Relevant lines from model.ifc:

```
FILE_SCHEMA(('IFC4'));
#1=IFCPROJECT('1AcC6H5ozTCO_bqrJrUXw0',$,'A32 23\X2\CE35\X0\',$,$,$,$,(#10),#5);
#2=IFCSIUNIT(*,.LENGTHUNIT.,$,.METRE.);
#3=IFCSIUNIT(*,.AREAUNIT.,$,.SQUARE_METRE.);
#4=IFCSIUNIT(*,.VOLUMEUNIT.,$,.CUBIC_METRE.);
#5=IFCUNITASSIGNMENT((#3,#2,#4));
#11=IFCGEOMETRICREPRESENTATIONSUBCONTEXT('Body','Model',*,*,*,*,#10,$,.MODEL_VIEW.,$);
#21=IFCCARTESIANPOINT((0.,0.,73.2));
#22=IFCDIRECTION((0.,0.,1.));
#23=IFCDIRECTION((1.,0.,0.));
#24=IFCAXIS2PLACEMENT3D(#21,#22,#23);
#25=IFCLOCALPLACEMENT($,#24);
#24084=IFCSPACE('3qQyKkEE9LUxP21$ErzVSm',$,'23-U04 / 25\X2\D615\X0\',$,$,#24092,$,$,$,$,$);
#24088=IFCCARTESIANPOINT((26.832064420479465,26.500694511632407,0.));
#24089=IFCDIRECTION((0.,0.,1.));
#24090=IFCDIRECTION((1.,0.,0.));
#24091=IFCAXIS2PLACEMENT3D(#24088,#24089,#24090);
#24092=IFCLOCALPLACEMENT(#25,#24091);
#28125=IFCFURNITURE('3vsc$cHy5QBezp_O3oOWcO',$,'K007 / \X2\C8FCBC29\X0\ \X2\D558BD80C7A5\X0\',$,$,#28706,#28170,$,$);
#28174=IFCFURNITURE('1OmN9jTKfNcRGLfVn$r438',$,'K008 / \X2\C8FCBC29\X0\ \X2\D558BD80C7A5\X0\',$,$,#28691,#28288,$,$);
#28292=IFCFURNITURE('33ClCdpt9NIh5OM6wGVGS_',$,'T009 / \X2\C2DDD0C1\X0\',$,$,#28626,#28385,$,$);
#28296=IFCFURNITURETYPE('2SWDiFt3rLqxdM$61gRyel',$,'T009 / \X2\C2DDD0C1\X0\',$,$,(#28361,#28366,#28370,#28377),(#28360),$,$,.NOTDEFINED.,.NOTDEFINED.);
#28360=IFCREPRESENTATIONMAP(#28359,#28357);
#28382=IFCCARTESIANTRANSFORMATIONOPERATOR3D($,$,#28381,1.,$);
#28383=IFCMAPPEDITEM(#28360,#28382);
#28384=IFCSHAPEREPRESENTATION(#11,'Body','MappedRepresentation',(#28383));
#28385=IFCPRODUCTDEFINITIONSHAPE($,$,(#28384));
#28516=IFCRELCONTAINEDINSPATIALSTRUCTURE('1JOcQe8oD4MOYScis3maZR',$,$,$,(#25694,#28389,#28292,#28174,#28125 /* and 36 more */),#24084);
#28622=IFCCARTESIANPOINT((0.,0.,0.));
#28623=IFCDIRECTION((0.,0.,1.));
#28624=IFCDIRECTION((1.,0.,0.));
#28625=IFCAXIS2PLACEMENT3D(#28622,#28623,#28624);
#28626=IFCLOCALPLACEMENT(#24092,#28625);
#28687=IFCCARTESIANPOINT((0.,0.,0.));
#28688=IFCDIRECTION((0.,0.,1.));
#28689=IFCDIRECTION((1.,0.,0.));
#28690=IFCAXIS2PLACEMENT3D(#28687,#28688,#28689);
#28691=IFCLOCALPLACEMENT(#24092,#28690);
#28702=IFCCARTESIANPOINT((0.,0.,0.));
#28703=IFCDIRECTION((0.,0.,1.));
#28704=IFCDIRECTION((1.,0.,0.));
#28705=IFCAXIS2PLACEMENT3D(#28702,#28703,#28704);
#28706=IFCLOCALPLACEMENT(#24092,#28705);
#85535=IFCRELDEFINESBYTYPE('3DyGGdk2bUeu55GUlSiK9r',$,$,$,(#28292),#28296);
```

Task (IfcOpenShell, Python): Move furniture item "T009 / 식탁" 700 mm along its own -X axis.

```python
import ifcopenshell
import ifcopenshell.api.geometry
import ifcopenshell.util.placement
import ifcopenshell.util.unit

model = ifcopenshell.open("model.ifc")
unit_scale = ifcopenshell.util.unit.calculate_unit_scale(model)

item = model.by_guid("33ClCdpt9NIh5OM6wGVGS_")
matrix = ifcopenshell.util.placement.get_local_placement(item.ObjectPlacement)
matrix[:3, 3] -= matrix[:3, 0] * 0.7 / unit_scale
ifcopenshell.api.geometry.edit_object_placement(model, product=item, matrix=matrix, is_si=False)

print(ifcopenshell.util.placement.get_local_placement(item.ObjectPlacement).round(3) + 0.0)

model.write("model_updated.ifc")
```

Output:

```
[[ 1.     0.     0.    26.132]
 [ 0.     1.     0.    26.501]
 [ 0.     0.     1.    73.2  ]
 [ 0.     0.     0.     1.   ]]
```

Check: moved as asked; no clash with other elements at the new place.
